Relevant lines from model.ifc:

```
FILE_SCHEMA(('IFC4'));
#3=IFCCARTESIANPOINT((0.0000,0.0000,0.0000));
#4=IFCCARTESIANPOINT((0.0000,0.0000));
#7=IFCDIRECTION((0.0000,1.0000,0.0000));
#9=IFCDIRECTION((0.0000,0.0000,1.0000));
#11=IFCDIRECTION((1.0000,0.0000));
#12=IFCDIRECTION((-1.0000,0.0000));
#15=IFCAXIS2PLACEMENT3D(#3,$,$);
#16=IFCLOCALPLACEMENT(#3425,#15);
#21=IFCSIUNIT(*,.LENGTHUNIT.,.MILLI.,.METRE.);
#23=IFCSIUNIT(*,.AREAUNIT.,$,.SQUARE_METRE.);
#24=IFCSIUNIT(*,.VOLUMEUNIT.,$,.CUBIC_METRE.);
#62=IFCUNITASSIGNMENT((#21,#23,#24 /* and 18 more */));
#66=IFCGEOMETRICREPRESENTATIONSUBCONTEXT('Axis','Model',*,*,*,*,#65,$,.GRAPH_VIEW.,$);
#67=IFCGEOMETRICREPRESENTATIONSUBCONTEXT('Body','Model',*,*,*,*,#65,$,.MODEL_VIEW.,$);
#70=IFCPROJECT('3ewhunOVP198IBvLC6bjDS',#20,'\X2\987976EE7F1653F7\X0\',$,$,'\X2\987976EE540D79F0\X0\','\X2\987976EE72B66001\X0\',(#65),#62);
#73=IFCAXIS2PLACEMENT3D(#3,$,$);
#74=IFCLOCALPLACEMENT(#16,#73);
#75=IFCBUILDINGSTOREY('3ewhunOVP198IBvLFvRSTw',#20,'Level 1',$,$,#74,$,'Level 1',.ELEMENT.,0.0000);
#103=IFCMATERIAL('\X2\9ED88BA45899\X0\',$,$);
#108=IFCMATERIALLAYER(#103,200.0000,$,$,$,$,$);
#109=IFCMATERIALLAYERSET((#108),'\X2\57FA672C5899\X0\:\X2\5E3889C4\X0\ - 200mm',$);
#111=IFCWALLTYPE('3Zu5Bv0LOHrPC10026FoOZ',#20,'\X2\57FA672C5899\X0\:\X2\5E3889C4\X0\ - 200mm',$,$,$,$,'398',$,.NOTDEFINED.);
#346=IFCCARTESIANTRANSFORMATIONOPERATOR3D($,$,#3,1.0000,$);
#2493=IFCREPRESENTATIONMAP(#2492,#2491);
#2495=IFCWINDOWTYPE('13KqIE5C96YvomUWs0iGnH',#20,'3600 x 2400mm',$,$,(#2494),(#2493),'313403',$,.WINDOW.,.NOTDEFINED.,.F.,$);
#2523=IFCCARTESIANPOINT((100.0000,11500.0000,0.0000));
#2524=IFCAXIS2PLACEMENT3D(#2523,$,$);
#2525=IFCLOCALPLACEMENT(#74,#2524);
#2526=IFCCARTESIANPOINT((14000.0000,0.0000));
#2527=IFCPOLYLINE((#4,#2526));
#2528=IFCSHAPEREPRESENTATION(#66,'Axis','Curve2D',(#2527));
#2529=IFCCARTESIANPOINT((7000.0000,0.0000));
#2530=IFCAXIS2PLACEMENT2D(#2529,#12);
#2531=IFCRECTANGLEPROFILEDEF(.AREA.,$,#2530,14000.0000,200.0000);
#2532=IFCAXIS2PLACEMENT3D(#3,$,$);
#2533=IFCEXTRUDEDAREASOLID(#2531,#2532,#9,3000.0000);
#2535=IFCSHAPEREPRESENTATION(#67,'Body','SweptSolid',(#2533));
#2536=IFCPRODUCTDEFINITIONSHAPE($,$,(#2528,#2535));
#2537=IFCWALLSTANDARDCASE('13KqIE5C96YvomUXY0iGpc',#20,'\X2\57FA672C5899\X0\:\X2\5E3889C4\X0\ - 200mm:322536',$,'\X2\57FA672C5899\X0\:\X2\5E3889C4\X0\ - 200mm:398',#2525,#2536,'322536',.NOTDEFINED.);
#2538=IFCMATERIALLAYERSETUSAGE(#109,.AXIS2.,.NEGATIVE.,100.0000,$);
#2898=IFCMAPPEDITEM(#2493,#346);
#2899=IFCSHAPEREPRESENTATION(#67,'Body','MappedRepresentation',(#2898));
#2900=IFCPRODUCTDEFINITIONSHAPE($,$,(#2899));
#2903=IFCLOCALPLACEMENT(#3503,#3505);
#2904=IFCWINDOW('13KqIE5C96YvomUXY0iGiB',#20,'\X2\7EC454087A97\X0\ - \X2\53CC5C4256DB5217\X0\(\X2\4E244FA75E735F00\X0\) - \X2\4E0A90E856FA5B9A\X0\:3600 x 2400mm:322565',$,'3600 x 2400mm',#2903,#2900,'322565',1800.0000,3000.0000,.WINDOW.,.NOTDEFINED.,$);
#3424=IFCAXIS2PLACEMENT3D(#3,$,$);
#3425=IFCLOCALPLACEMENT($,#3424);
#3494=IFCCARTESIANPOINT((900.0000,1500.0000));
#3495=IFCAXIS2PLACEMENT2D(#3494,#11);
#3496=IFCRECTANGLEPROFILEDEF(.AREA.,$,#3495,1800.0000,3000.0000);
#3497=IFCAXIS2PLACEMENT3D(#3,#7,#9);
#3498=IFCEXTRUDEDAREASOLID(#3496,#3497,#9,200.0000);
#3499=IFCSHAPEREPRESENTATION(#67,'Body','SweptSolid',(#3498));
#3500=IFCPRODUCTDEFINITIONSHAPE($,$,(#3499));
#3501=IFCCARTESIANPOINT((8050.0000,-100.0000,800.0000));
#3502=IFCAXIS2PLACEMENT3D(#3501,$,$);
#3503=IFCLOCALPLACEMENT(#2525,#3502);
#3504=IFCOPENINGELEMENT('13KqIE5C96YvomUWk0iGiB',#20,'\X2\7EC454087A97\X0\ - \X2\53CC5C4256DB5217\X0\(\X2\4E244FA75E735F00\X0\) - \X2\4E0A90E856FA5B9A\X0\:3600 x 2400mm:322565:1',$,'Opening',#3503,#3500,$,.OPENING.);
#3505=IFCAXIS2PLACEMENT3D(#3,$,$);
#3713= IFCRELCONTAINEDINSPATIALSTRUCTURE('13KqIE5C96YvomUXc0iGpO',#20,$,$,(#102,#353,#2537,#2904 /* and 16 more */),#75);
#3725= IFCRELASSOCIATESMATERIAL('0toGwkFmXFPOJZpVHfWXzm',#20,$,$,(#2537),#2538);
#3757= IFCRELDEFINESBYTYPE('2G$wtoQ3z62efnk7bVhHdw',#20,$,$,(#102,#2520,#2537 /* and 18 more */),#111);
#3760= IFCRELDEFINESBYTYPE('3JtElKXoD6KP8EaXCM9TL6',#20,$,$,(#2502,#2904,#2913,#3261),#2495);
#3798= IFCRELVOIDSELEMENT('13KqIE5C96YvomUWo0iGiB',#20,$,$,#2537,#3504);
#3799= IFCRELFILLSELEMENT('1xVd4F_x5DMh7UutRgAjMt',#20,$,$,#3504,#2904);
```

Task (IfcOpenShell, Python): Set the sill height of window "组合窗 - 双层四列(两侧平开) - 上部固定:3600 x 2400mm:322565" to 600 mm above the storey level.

```python
import numpy as np
import ifcopenshell
import ifcopenshell.api.geometry
import ifcopenshell.geom
import ifcopenshell.util.element
import ifcopenshell.util.placement
import ifcopenshell.util.shape
import ifcopenshell.util.unit

model = ifcopenshell.open("model.ifc")
unit_scale = ifcopenshell.util.unit.calculate_unit_scale(model)

window = model.by_guid("13KqIE5C96YvomUXY0iGiB")
opening = window.FillsVoids[0].RelatingOpeningElement
storey = ifcopenshell.util.element.get_container(window, ifc_class="IfcBuildingStorey")
level = ifcopenshell.util.placement.get_local_placement(storey.ObjectPlacement)[2, 3]

# The opening's origin need not be at the sill, so measure its lowest point.
shape = ifcopenshell.geom.create_shape(ifcopenshell.geom.settings(), opening)
bottom = ifcopenshell.util.shape.get_shape_bottom_elevation(shape, shape.geometry) / unit_scale
dz = level + 0.6 / unit_scale - bottom

shift = np.array([0.0, 0.0, dz])
# The window is placed relative to its opening, so it follows when the opening moves.
matrix = ifcopenshell.util.placement.get_local_placement(opening.ObjectPlacement)
matrix[:3, 3] += shift
ifcopenshell.api.geometry.edit_object_placement(
    model, product=opening, matrix=matrix, is_si=False, should_transform_children=True
)

print(f"moved by {dz * unit_scale:+.3f} m")

model.write("model_v2.ifc")
```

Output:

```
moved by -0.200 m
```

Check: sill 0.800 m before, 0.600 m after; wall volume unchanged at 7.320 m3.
